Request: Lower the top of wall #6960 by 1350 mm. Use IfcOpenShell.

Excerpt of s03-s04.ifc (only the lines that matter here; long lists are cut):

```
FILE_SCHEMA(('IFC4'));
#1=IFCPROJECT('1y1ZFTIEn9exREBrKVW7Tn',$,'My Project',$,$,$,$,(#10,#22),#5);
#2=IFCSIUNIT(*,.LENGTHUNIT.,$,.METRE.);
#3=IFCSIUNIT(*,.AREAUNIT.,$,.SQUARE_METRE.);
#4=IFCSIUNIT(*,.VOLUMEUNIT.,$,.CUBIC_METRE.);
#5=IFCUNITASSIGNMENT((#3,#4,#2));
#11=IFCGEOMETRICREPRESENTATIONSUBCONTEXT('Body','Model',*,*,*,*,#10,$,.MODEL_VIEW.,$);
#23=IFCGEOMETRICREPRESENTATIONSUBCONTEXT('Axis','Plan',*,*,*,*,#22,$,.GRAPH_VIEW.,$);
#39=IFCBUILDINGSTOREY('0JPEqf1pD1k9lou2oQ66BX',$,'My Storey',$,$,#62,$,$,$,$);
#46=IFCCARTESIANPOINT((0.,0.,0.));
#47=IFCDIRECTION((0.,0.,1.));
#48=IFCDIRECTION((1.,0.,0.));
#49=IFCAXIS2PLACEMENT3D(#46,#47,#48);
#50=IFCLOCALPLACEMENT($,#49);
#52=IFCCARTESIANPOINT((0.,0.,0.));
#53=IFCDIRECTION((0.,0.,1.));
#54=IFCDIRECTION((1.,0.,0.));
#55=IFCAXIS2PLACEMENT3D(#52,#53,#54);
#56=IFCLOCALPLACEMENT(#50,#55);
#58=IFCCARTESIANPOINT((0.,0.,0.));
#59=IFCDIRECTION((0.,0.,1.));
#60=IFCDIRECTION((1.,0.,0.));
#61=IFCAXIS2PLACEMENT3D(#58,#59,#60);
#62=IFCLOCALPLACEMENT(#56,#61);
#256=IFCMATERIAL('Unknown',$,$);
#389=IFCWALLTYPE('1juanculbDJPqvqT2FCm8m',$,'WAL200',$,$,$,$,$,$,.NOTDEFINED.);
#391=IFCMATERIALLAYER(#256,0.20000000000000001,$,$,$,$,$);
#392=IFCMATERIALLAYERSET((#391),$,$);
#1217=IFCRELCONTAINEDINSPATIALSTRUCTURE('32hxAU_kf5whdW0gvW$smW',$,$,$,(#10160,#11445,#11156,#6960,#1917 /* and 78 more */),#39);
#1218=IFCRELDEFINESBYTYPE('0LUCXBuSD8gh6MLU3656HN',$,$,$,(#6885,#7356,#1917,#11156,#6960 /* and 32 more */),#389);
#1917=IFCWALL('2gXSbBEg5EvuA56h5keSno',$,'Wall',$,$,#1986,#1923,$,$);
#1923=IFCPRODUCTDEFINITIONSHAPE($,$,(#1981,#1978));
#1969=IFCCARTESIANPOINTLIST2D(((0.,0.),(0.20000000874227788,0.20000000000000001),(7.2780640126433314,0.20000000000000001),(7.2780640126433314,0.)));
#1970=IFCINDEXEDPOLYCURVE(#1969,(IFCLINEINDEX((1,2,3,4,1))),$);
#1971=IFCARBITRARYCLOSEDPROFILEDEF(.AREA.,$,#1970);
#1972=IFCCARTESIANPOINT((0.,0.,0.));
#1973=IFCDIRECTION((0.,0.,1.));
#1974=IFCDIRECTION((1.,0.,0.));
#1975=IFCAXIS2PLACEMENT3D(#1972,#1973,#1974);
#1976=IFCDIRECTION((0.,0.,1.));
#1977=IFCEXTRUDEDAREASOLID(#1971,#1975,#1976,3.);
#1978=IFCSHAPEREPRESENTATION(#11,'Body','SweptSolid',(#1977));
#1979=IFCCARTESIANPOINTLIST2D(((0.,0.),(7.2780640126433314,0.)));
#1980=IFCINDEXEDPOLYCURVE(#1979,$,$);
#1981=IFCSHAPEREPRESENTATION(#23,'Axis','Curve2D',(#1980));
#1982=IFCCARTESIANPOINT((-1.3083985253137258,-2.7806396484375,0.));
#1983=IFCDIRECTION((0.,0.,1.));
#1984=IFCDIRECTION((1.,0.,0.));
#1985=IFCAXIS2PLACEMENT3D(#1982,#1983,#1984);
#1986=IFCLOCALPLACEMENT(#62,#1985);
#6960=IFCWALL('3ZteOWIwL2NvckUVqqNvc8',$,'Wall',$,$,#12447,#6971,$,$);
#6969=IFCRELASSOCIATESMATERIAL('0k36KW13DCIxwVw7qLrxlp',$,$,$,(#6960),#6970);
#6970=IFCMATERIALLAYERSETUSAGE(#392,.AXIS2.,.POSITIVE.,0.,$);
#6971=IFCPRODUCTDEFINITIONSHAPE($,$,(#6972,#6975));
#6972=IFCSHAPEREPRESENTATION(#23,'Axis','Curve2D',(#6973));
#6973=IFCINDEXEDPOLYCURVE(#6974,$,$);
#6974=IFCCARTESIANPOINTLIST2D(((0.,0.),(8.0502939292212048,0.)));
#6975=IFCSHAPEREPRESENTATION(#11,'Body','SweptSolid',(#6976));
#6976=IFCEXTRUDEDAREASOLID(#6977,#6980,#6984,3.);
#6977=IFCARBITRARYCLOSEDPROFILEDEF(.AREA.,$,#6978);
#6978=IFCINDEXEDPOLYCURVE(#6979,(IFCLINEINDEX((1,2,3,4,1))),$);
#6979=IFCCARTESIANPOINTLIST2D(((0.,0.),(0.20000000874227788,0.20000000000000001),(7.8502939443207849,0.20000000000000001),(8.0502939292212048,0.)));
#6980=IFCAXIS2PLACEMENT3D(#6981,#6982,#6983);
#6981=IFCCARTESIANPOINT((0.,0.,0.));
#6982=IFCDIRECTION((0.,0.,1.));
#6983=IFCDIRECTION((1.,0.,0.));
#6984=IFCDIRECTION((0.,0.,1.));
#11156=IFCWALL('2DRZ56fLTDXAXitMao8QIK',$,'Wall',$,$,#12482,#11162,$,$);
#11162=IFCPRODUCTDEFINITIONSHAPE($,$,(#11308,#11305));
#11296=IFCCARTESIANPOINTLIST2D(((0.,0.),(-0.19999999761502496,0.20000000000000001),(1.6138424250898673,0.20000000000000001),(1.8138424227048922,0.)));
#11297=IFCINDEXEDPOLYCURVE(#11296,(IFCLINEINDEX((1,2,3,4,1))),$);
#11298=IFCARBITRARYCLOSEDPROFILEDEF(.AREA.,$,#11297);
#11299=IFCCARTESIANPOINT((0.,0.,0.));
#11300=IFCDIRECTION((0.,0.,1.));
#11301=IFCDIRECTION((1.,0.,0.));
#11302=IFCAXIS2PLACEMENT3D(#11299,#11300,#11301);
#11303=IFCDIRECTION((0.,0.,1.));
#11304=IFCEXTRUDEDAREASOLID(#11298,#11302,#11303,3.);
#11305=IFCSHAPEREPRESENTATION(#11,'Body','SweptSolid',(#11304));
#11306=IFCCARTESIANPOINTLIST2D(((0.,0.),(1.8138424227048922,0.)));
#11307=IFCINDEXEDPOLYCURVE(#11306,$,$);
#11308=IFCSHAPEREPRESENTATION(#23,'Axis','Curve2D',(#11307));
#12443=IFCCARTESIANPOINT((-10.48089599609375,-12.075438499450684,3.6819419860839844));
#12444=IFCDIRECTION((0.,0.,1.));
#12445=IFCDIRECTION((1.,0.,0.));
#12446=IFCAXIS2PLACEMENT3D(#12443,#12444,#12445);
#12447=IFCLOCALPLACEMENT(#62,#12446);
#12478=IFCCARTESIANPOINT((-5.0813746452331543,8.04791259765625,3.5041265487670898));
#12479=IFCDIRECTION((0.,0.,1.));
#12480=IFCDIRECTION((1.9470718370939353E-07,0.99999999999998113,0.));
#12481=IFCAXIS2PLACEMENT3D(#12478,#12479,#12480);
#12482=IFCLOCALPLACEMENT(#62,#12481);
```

```python
import ifcopenshell
import ifcopenshell.geom
import ifcopenshell.util.representation
import ifcopenshell.util.shape

model = ifcopenshell.open("s03-s04.ifc")
settings = ifcopenshell.geom.settings()


def volume(element):
    """Net volume in cubic metres, openings subtracted."""
    shape = ifcopenshell.geom.create_shape(settings, element)
    return ifcopenshell.util.shape.get_volume(shape.geometry)


wall = model.by_guid("3ZteOWIwL2NvckUVqqNvc8")
before = volume(wall)

body = ifcopenshell.util.representation.get_representation(wall, "Model", "Body")
solid = body.Items[0]
old_height = solid.Depth
solid.Depth -= 1.35
after = volume(wall)

print(f"height {old_height:g} -> {solid.Depth:g}, volume {before:.3f} -> {after:.3f} m3")

model.write("s03-s04-out.ifc")
```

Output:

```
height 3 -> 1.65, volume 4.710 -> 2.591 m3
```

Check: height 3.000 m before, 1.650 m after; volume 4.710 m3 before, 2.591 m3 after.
